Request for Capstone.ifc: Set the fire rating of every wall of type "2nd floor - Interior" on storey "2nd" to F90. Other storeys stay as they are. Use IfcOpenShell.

First a look at what the model holds.

```python
import ifcopenshell
import ifcopenshell.util.element

model = ifcopenshell.open("Capstone.ifc")
print(model.schema)
storey = next(s for s in model.by_type("IfcBuildingStorey") if s.Name == "2nd")
walls = [e for e in ifcopenshell.util.element.get_decomposition(storey) if e.is_a("IfcWall")]
seen = {}
for e in walls:
    element_type = ifcopenshell.util.element.get_type(e)
    key = (element_type.Name if element_type != e and element_type else None, ifcopenshell.util.element.get_pset(e, "Pset_WallCommon", "FireRating"))
    seen[key] = seen.get(key, 0) + 1
for (name, value), count in sorted(seen.items(), key=str):
    print(count, "x", name, "|", value)
```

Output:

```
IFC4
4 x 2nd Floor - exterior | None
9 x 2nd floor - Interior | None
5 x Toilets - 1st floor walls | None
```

```python
import ifcopenshell
import ifcopenshell.api.pset
import ifcopenshell.util.element

model = ifcopenshell.open("Capstone.ifc")

storey = next(s for s in model.by_type("IfcBuildingStorey") if s.Name == "2nd")
walls = [e for e in ifcopenshell.util.element.get_decomposition(storey) if e.is_a("IfcWall")]

count = 0
for e in walls:
    element_type = ifcopenshell.util.element.get_type(e)
    if element_type in (None, e) or element_type.Name != "2nd floor - Interior":
        continue
    # add_pset returns the element's existing set when there is one.
    pset = ifcopenshell.api.pset.add_pset(model, product=e, name="Pset_WallCommon")
    ifcopenshell.api.pset.edit_pset(model, pset=pset, properties={"FireRating": "F90"})
    count += 1

print(count, "walls updated")

model.write("Capstone_v2.ifc")
```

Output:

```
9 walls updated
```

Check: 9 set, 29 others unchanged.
